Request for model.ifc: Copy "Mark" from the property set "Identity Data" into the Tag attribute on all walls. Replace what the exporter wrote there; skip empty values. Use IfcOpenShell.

First a look at what the model holds.

```python
import ifcopenshell
import ifcopenshell.util.element

model = ifcopenshell.open("model.ifc")
print(model.schema)
walls = model.by_type("IfcWall")
print(len(walls), "walls")
for e in walls[:8]:
    source = ifcopenshell.util.element.get_pset(e, "Identity Data", "Mark")
    target = e.Tag
    print(e.id(), repr(source), repr(target), sep=" | ")
```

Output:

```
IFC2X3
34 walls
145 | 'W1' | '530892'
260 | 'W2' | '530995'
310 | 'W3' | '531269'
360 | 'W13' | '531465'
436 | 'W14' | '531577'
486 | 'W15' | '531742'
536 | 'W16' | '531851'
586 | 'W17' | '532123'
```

```python
import ifcopenshell
import ifcopenshell.util.element

model = ifcopenshell.open("model.ifc")

count = 0
for e in model.by_type("IfcWall"):
    value = ifcopenshell.util.element.get_pset(e, "Identity Data", "Mark")
    current = e.Tag
    if not value or not value.strip() or current == value:
        continue
    e.Tag = value
    count += 1

print(count, "walls updated")

model.write("model_rev.ifc")
```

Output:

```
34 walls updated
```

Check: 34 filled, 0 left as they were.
